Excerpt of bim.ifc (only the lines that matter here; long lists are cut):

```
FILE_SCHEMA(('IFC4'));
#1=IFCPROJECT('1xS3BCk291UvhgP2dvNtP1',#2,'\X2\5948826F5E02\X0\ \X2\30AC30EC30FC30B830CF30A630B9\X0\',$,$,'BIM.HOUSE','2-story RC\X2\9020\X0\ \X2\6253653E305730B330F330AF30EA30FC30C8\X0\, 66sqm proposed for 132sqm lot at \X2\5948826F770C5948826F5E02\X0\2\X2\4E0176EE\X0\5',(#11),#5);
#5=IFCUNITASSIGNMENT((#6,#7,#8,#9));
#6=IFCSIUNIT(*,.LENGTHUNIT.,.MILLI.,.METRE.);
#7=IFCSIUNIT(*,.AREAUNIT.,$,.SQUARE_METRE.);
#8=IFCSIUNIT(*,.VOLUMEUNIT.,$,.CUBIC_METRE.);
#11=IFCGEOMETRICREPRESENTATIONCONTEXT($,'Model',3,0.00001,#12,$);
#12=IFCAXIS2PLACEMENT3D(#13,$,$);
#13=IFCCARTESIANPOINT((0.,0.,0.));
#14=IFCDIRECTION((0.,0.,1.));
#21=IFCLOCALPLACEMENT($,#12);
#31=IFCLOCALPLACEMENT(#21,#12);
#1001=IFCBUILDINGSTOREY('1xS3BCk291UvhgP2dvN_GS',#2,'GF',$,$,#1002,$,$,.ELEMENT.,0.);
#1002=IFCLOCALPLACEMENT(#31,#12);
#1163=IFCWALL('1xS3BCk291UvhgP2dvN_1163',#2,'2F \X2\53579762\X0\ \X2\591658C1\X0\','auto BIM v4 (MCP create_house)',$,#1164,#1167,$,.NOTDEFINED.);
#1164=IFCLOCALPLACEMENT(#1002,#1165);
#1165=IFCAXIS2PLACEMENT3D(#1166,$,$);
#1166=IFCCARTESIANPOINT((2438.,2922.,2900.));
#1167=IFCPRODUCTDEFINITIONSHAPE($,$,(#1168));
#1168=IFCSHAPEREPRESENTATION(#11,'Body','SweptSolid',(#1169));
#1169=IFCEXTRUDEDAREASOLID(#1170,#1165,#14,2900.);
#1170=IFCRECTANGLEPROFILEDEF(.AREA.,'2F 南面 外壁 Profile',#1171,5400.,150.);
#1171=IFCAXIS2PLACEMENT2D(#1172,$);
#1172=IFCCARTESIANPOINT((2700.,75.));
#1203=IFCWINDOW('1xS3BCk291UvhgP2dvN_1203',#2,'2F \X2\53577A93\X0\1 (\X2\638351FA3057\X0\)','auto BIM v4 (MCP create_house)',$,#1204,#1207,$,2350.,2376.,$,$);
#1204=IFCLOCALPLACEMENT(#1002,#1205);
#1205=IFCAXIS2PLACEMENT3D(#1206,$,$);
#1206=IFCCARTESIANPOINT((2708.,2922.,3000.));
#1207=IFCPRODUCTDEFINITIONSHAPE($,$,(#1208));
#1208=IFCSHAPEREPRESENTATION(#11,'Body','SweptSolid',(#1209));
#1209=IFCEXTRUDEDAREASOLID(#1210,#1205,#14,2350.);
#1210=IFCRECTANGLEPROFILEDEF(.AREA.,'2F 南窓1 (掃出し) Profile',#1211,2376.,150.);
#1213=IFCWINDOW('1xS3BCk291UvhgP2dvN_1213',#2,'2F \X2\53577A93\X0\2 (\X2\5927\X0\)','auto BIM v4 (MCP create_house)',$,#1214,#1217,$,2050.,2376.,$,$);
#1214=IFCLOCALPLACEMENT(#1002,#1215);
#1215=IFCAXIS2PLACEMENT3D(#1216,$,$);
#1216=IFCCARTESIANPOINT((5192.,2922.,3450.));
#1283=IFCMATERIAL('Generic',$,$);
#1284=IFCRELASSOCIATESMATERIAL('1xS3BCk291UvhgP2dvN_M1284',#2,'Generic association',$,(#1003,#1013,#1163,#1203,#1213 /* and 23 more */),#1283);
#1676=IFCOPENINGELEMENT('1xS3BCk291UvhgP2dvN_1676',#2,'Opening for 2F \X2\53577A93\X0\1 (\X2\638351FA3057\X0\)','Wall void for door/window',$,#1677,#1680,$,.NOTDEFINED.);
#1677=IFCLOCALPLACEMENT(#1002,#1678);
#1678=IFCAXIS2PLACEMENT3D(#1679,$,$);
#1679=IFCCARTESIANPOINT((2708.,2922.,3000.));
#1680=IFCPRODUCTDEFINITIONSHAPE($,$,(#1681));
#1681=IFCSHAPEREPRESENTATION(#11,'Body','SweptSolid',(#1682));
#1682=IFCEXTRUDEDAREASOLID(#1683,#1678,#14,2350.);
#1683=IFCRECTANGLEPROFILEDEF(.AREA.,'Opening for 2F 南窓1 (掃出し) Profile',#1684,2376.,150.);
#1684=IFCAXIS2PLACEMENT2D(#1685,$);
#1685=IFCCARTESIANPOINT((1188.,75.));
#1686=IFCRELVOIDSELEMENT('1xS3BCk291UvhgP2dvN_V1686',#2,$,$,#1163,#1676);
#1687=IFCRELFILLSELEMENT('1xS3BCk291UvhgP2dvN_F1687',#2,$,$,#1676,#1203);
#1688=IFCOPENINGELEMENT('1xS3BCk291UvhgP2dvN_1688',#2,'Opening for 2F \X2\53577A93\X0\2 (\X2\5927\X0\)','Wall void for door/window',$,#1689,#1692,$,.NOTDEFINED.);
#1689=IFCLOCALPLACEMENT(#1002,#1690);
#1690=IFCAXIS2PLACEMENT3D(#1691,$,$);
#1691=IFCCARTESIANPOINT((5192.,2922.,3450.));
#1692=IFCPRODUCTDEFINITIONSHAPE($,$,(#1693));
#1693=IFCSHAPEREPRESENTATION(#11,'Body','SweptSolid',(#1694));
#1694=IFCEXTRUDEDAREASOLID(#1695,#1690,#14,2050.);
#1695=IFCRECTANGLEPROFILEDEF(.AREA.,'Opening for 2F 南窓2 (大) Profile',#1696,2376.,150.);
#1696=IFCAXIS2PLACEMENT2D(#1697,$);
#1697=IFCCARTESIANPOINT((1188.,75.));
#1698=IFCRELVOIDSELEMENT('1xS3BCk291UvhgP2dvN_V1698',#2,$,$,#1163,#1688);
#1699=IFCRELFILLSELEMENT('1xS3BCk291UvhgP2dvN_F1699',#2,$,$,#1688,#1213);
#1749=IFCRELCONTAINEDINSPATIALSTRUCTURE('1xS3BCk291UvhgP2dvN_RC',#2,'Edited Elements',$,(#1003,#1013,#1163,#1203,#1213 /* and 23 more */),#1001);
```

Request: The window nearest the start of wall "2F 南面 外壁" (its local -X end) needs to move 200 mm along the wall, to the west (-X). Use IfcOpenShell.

```python
import ifcopenshell
import ifcopenshell.api.geometry
import ifcopenshell.util.placement
import ifcopenshell.util.unit

model = ifcopenshell.open("bim.ifc")
unit_scale = ifcopenshell.util.unit.calculate_unit_scale(model)

window = model.by_id(1203)
opening = window.FillsVoids[0].RelatingOpeningElement
wall = opening.VoidsElements[0].RelatingBuildingElement

wall_matrix = ifcopenshell.util.placement.get_local_placement(wall.ObjectPlacement)
shift = wall_matrix[:3, 0] * -0.2 / unit_scale
before = ifcopenshell.util.placement.get_local_placement(window.ObjectPlacement)[:3, 3].copy()

# The window is not placed relative to its opening, so move both.
for product in (opening, window):
    matrix = ifcopenshell.util.placement.get_local_placement(product.ObjectPlacement)
    matrix[:3, 3] += shift
    ifcopenshell.api.geometry.edit_object_placement(model, product=product, matrix=matrix, is_si=False)

after = ifcopenshell.util.placement.get_local_placement(window.ObjectPlacement)[:3, 3]
print("window moved by", (after - before).round(3) + 0.0)

model.write("bim_v2.ifc")
```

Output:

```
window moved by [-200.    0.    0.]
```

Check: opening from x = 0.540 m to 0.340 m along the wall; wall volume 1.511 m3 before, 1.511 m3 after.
